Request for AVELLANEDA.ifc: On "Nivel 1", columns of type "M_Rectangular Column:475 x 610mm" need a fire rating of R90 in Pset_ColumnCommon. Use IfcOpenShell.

First a look at what the model holds.

```python
import ifcopenshell
import ifcopenshell.util.element

model = ifcopenshell.open("AVELLANEDA.ifc")
print(model.schema)
storey = next(s for s in model.by_type("IfcBuildingStorey") if s.Name == "Nivel 1")
columns = [e for e in ifcopenshell.util.element.get_decomposition(storey) if e.is_a("IfcColumn")]
seen = {}
for e in columns:
    element_type = ifcopenshell.util.element.get_type(e)
    key = (element_type.Name if element_type != e and element_type else None, ifcopenshell.util.element.get_pset(e, "Pset_ColumnCommon", "FireRating"))
    seen[key] = seen.get(key, 0) + 1
for (name, value), count in sorted(seen.items(), key=str):
    print(count, "x", name, "|", value)
```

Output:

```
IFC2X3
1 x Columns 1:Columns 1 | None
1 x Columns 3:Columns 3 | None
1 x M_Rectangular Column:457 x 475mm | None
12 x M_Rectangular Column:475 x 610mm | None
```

```python
import ifcopenshell
import ifcopenshell.api.pset
import ifcopenshell.util.element

model = ifcopenshell.open("AVELLANEDA.ifc")

storey = next(s for s in model.by_type("IfcBuildingStorey") if s.Name == "Nivel 1")
columns = [e for e in ifcopenshell.util.element.get_decomposition(storey) if e.is_a("IfcColumn")]

count = 0
for e in columns:
    element_type = ifcopenshell.util.element.get_type(e)
    if element_type in (None, e) or element_type.Name != "M_Rectangular Column:475 x 610mm":
        continue
    # add_pset returns the element's existing set when there is one.
    pset = ifcopenshell.api.pset.add_pset(model, product=e, name="Pset_ColumnCommon")
    ifcopenshell.api.pset.edit_pset(model, pset=pset, properties={"FireRating": "R90"})
    count += 1

print(count, "columns updated")

model.write("AVELLANEDA_updated.ifc")
```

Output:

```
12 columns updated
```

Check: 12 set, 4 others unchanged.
